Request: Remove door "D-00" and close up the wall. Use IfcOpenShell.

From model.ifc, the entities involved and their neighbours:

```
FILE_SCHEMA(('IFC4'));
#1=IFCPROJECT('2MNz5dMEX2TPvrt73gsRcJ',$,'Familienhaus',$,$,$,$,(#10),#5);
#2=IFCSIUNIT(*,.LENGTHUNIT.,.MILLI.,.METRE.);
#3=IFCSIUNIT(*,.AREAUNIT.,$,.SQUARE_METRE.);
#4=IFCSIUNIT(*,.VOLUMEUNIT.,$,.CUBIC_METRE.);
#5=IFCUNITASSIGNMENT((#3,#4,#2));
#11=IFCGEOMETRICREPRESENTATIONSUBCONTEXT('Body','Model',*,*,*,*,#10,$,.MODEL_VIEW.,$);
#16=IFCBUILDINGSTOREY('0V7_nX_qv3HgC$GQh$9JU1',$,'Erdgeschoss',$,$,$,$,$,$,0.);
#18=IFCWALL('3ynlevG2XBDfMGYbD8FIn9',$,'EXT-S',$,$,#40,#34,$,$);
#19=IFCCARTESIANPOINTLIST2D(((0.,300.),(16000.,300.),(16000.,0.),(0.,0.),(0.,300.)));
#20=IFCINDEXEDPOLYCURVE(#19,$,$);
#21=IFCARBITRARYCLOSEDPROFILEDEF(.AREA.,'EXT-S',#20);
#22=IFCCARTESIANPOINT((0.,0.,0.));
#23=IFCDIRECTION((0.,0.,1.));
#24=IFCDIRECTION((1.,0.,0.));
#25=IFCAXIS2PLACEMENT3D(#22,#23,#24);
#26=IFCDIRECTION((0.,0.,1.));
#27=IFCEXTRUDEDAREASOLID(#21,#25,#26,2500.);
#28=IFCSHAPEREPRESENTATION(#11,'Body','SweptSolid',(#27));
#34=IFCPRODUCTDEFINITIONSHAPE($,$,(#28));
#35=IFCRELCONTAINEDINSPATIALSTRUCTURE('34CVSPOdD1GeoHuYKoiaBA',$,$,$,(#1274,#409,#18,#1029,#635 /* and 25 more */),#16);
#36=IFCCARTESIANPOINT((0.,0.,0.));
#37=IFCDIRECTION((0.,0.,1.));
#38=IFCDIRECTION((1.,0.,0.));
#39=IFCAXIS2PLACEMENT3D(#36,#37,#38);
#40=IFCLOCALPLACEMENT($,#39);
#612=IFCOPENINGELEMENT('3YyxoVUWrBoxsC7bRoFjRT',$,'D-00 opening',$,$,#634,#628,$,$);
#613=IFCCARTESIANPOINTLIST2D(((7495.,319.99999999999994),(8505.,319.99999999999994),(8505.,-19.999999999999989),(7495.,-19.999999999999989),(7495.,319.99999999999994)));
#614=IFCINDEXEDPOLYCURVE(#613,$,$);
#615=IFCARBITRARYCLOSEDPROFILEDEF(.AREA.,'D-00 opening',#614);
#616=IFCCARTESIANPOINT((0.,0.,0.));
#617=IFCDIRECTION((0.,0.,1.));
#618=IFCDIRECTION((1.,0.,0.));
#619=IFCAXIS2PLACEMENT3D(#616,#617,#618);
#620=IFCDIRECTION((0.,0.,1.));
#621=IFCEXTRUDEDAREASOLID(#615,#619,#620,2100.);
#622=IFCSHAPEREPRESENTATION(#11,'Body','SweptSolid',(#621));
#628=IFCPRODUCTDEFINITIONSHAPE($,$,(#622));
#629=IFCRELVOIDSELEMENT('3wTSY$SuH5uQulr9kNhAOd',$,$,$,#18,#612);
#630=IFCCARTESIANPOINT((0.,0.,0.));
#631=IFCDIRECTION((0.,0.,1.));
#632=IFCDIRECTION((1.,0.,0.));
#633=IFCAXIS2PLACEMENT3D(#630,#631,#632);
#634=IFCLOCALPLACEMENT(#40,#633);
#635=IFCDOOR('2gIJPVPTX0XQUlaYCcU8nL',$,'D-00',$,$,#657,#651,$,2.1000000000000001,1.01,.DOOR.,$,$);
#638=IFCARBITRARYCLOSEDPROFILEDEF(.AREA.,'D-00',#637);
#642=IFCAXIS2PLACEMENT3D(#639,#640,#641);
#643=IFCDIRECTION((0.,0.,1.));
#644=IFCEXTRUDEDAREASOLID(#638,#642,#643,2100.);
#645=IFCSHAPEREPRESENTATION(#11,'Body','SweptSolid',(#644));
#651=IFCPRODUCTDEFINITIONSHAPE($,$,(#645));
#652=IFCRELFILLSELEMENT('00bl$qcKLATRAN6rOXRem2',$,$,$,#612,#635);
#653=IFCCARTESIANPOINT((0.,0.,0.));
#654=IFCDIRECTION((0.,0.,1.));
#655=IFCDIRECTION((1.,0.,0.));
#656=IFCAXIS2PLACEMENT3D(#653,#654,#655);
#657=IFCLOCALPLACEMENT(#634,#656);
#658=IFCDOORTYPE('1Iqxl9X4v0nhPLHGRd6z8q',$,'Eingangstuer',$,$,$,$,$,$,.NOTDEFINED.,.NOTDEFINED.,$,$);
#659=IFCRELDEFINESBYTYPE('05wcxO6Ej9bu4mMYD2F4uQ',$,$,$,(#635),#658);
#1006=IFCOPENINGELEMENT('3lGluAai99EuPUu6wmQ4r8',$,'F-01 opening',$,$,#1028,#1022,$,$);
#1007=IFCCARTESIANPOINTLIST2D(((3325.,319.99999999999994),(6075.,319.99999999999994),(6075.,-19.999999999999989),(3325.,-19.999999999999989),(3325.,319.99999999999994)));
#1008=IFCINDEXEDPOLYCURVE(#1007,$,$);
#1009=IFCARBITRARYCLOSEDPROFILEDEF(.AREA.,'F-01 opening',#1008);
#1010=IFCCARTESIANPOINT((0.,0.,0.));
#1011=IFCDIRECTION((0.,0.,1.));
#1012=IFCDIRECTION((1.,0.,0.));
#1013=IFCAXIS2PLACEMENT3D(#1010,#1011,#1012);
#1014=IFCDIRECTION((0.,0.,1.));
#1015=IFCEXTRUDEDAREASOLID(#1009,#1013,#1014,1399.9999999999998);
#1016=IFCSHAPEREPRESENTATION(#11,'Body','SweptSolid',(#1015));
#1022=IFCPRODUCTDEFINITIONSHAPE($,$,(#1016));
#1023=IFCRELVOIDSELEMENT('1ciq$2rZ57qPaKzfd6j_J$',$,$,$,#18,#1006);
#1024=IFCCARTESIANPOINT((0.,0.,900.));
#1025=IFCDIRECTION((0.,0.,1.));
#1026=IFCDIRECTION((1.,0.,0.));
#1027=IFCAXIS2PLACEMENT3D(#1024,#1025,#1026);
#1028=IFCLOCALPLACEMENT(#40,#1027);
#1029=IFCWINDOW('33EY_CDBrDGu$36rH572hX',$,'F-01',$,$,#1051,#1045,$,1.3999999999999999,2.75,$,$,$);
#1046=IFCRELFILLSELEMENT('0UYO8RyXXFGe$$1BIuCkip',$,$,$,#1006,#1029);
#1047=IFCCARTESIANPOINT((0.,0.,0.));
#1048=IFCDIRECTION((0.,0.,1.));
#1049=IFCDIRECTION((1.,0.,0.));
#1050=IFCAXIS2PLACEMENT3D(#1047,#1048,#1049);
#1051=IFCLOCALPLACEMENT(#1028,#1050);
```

```python
import ifcopenshell
import ifcopenshell.api.feature
import ifcopenshell.api.root
import ifcopenshell.geom
import ifcopenshell.util.shape

model = ifcopenshell.open("model.ifc")
settings = ifcopenshell.geom.settings()


def volume(element):
    """Net volume in cubic metres, openings subtracted."""
    shape = ifcopenshell.geom.create_shape(settings, element)
    return ifcopenshell.util.shape.get_volume(shape.geometry)


door = model.by_id(635)
opening = door.FillsVoids[0].RelatingOpeningElement
wall = opening.VoidsElements[0].RelatingBuildingElement
before = volume(wall)

ifcopenshell.api.root.remove_product(model, product=door)
ifcopenshell.api.feature.remove_feature(model, feature=opening)

after = volume(wall)

print(f"wall volume {before:.3f} -> {after:.3f} m3")

model.write("model_rev.ifc")
```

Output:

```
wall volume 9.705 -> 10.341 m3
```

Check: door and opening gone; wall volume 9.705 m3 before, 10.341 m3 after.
